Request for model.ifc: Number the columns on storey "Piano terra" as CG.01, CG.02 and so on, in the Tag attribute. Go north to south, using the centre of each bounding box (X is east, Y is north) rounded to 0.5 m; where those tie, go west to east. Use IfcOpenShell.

First a look at what the model holds.

```python
import ifcopenshell
import ifcopenshell.util.element
import ifcopenshell.util.placement

model = ifcopenshell.open("model.ifc")
print(model.schema)
storey = next(s for s in model.by_type("IfcBuildingStorey") if s.Name == "Piano terra")
columns = [e for e in ifcopenshell.util.element.get_decomposition(storey) if e.is_a("IfcColumn")]
for e in sorted(columns, key=lambda e: e.id()):
    origin = ifcopenshell.util.placement.get_local_placement(e.ObjectPlacement)[:3, 3]
    print(e.id(), e.Tag, e.Name, origin.round(2) + 0.0, sep=" | ")
```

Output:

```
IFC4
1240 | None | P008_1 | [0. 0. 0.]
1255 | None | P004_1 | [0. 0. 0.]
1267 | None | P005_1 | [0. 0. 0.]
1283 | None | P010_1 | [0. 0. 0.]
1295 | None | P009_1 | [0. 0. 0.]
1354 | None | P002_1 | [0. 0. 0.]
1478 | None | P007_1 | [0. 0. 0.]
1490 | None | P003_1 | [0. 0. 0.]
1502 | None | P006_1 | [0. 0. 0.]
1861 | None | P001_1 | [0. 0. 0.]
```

```python
import ifcopenshell
import ifcopenshell.geom
import ifcopenshell.util.element
import ifcopenshell.util.shape

model = ifcopenshell.open("model.ifc")
settings = ifcopenshell.geom.settings()
settings.set("use-world-coords", True)


def centre(element):
    shape = ifcopenshell.geom.create_shape(settings, element)
    return ifcopenshell.util.shape.get_bbox_centroid(shape.geometry)


storey = next(s for s in model.by_type("IfcBuildingStorey") if s.Name == "Piano terra")
columns = [e for e in ifcopenshell.util.element.get_decomposition(storey) if e.is_a("IfcColumn")]

# Insertion points can sit at a corner or the storey origin, so sort by the geometry (in metres).
centres = {e: centre(e) for e in columns}
columns.sort(key=lambda e: (-round(centres[e][1] / 0.5), centres[e][0]))

for i, e in enumerate(columns, start=1):
    number = f"CG.{i:02d}"
    e.Tag = number
    print(e.id(), number)

model.write("model_v2.ifc")
```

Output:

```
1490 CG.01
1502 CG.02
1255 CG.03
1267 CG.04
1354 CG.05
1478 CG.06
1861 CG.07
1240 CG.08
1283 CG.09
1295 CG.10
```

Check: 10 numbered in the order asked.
